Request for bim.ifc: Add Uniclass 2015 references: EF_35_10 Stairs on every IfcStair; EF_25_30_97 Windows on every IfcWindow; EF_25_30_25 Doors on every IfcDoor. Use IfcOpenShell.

First a look at what the model holds.

```python
import ifcopenshell

model = ifcopenshell.open("bim.ifc")
print(model.schema)
print("classifications:", [c.Name for c in model.by_type("IfcClassification")])
for ifc_class in ("IfcDoor", "IfcRoof", "IfcStair", "IfcWall", "IfcWindow"):
    print(ifc_class, len(model.by_type(ifc_class)))
```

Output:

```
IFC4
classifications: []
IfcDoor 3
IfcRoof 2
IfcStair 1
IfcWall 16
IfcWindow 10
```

```python
import ifcopenshell
import ifcopenshell.api.classification

model = ifcopenshell.open("bim.ifc")

system = ifcopenshell.api.classification.add_classification(model, classification="Uniclass 2015")

codes = {
    "IfcStair": ("EF_35_10", "Stairs"),
    "IfcWindow": ("EF_25_30_97", "Windows"),
    "IfcDoor": ("EF_25_30_25", "Doors"),
}
for ifc_class, (code, name) in codes.items():
    products = model.by_type(ifc_class)
    ifcopenshell.api.classification.add_reference(
        model, products=products, classification=system, identification=code, name=name
    )
    print(code, len(products))

model.write("bim_rev.ifc")
```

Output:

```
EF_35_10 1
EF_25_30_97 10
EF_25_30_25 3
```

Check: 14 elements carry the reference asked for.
